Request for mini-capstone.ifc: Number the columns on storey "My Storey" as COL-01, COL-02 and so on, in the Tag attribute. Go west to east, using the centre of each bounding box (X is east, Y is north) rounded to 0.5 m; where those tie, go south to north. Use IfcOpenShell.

First a look at what the model holds.

```python
import ifcopenshell
import ifcopenshell.util.element
import ifcopenshell.util.placement

model = ifcopenshell.open("mini-capstone.ifc")
print(model.schema)
storey = next(s for s in model.by_type("IfcBuildingStorey") if s.Name == "My Storey")
columns = [e for e in ifcopenshell.util.element.get_decomposition(storey) if e.is_a("IfcColumn")]
for e in sorted(columns, key=lambda e: e.id()):
    origin = ifcopenshell.util.placement.get_local_placement(e.ObjectPlacement)[:3, 3]
    print(e.id(), e.Tag, e.Name, origin.round(2) + 0.0, sep=" | ")
```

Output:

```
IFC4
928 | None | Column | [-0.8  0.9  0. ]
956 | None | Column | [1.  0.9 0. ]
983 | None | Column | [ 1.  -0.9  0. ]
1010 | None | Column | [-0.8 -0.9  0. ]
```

```python
import ifcopenshell
import ifcopenshell.geom
import ifcopenshell.util.element
import ifcopenshell.util.shape

model = ifcopenshell.open("mini-capstone.ifc")
settings = ifcopenshell.geom.settings()
settings.set("use-world-coords", True)


def centre(element):
    shape = ifcopenshell.geom.create_shape(settings, element)
    return ifcopenshell.util.shape.get_bbox_centroid(shape.geometry)


storey = next(s for s in model.by_type("IfcBuildingStorey") if s.Name == "My Storey")
columns = [e for e in ifcopenshell.util.element.get_decomposition(storey) if e.is_a("IfcColumn")]

# Insertion points can sit at a corner or the storey origin, so sort by the geometry (in metres).
centres = {e: centre(e) for e in columns}
columns.sort(key=lambda e: (round(centres[e][0] / 0.5), centres[e][1]))

for i, e in enumerate(columns, start=1):
    number = f"COL-{i:02d}"
    e.Tag = number
    print(e.id(), number)

model.write("mini-capstone_updated.ifc")
```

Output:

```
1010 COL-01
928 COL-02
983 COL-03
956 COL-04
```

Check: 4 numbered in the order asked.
